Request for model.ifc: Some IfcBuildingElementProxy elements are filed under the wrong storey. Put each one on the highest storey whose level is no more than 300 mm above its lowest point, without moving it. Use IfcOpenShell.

First a look at what the model holds.

```python
import ifcopenshell
import ifcopenshell.util.element
import ifcopenshell.util.placement

model = ifcopenshell.open("model.ifc")
print(model.schema)
for storey in model.by_type("IfcBuildingStorey"):
    level = ifcopenshell.util.placement.get_storey_elevation(storey)
    count = sum(e.is_a("IfcBuildingElementProxy") for e in ifcopenshell.util.element.get_contained(storey))
    print(storey.id(), storey.Name, round(level, 3), count, sep=" | ")
```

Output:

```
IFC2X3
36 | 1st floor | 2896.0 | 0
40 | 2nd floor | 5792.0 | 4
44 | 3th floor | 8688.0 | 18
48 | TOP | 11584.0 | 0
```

```python
import ifcopenshell
import ifcopenshell.api.spatial
import ifcopenshell.geom
import ifcopenshell.util.element
import ifcopenshell.util.placement
import ifcopenshell.util.shape
import ifcopenshell.util.unit

model = ifcopenshell.open("model.ifc")
unit_scale = ifcopenshell.util.unit.calculate_unit_scale(model)
settings = ifcopenshell.geom.settings()

levels = sorted(
    ((ifcopenshell.util.placement.get_storey_elevation(s) * unit_scale, s) for s in model.by_type("IfcBuildingStorey")),
    key=lambda pair: pair[0],
)

for e in model.by_type("IfcBuildingElementProxy"):
    current = e.ContainedInStructure[0].RelatingStructure if e.ContainedInStructure else None
    if current is None or not current.is_a("IfcBuildingStorey"):
        continue
    shape = ifcopenshell.geom.create_shape(settings, e)
    bottom = ifcopenshell.util.shape.get_shape_bottom_elevation(shape, shape.geometry)
    below = [s for level, s in levels if level <= bottom + 0.3]
    storey = below[-1] if below else levels[0][1]
    if storey != current:
        # assign_container keeps the world position.
        ifcopenshell.api.spatial.assign_container(model, products=[e], relating_structure=storey)
        print(e.id(), current.Name, "->", storey.Name)

model.write("model-out.ifc")
```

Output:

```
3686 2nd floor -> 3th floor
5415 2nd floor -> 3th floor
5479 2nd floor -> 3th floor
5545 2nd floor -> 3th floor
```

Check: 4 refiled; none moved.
